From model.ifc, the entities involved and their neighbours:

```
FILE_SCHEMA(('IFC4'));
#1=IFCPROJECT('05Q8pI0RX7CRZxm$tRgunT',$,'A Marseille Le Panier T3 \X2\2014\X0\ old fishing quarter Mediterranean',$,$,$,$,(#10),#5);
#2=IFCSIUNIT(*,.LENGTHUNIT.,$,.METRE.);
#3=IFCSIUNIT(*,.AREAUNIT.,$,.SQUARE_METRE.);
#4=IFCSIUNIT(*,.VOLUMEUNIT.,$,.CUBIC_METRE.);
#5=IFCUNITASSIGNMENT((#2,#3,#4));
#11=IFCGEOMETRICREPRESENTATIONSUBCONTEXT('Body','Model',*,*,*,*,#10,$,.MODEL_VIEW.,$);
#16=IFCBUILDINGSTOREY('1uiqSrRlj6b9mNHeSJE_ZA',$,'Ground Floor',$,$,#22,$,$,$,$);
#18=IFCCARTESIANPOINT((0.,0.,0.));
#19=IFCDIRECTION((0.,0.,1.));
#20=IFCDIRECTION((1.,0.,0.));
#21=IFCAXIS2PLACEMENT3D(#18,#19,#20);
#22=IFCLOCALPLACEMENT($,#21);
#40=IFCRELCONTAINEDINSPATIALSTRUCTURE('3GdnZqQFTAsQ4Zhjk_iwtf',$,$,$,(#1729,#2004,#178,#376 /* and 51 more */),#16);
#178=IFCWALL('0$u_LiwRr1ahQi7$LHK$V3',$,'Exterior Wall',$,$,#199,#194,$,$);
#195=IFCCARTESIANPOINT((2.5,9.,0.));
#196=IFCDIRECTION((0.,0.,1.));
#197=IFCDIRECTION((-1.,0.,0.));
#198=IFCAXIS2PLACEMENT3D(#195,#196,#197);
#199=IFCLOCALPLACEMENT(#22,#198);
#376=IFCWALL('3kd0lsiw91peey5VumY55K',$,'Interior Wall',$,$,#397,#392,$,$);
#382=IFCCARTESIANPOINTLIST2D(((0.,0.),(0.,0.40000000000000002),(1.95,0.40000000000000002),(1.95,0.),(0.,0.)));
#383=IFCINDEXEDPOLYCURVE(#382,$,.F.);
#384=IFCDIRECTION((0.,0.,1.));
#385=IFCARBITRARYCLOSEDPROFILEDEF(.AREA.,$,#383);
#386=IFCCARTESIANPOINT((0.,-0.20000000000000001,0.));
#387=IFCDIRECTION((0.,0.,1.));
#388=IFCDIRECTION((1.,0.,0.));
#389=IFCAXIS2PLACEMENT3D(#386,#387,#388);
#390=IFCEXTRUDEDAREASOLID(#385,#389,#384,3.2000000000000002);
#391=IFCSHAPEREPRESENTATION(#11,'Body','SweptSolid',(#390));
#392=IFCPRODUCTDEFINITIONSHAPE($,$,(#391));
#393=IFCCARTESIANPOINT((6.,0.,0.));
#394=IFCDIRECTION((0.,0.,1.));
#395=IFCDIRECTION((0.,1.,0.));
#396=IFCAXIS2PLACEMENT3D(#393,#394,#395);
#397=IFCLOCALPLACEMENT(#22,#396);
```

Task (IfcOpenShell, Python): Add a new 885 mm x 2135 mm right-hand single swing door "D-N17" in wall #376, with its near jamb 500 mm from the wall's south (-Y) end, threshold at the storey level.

```python
import numpy as np
import ifcopenshell
import ifcopenshell.api.feature
import ifcopenshell.api.geometry
import ifcopenshell.api.root
import ifcopenshell.api.spatial
import ifcopenshell.geom
import ifcopenshell.util.element
import ifcopenshell.util.placement
import ifcopenshell.util.representation
import ifcopenshell.util.shape
import ifcopenshell.util.unit

model = ifcopenshell.open("model.ifc")
unit_scale = ifcopenshell.util.unit.calculate_unit_scale(model)
settings = ifcopenshell.geom.settings()


def volume(element):
    """Net volume in cubic metres, openings subtracted."""
    shape = ifcopenshell.geom.create_shape(settings, element)
    return ifcopenshell.util.shape.get_volume(shape.geometry)


wall = model.by_guid("3kd0lsiw91peey5VumY55K")
storey = ifcopenshell.util.element.get_container(wall, ifc_class="IfcBuildingStorey")
context = ifcopenshell.util.representation.get_context(model, "Model", "Body", "MODEL_VIEW")
before = volume(wall)

width, height, from_end, sill = 0.885, 2.135, 0.5, 0.0  # metres

# The wall runs along its own X axis, and the end named is its -X end.
wall_shape = ifcopenshell.geom.create_shape(settings, wall)
x, y, z = ifcopenshell.util.shape.get_vertices(wall_shape.geometry).T
start = x.min() + from_end
face, thickness = float(y.min()), float(y.max() - y.min())
wall_matrix = ifcopenshell.util.placement.get_local_placement(wall.ObjectPlacement)
level = ifcopenshell.util.placement.get_local_placement(storey.ObjectPlacement)[2, 3]


def in_wall(x, y):
    """Placement at x, y metres in the wall's axes, at sill height."""
    matrix = wall_matrix.copy()
    matrix[:, 3] = wall_matrix @ np.array([x / unit_scale, y / unit_scale, 0.0, 1.0])
    matrix[2, 3] = level + sill / unit_scale
    return matrix


# Opening: a box that overshoots both wall faces by 50 mm.
opening = ifcopenshell.api.root.create_entity(model, ifc_class="IfcOpeningElement", predefined_type="OPENING")
box = ifcopenshell.api.geometry.add_wall_representation(
    model, context=context, length=width, height=height, thickness=thickness + 0.1
)
ifcopenshell.api.geometry.assign_representation(model, product=opening, representation=box)
ifcopenshell.api.geometry.edit_object_placement(model, product=opening, matrix=in_wall(start, face - 0.05), is_si=False)
ifcopenshell.api.feature.add_feature(model, feature=opening, element=wall)

door = ifcopenshell.api.root.create_entity(model, ifc_class="IfcDoor", name="D-N17", predefined_type="DOOR")
door.OverallWidth, door.OverallHeight = width / unit_scale, height / unit_scale
door.OperationType = "SINGLE_SWING_RIGHT"
body = ifcopenshell.api.geometry.add_door_representation(
    model,
    context=context,
    overall_width=door.OverallWidth,
    overall_height=door.OverallHeight,
    operation_type="SINGLE_SWING_RIGHT",
    lining_properties={"LiningDepth": thickness / unit_scale, "ThresholdDepth": thickness / unit_scale},
)
ifcopenshell.api.geometry.assign_representation(model, product=door, representation=body)
ifcopenshell.api.spatial.assign_container(model, products=[door], relating_structure=storey)
ifcopenshell.api.feature.add_filling(model, opening=opening, element=door)

# The lining spans the wall, so the door starts at the wall face.
ifcopenshell.api.geometry.edit_object_placement(model, product=door, matrix=in_wall(start, face), is_si=False)

after = volume(wall)

print(f"wall volume {before:.3f} -> {after:.3f} m3")

model.write("model-out.ifc")
```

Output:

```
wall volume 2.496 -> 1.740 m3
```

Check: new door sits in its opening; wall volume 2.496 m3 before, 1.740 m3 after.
